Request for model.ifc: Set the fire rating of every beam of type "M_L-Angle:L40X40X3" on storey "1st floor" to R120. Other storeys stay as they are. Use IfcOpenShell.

First a look at what the model holds.

```python
import ifcopenshell
import ifcopenshell.util.element

model = ifcopenshell.open("model.ifc")
print(model.schema)
storey = next(s for s in model.by_type("IfcBuildingStorey") if s.Name == "1st floor")
beams = [e for e in ifcopenshell.util.element.get_decomposition(storey) if e.is_a("IfcBeam")]
seen = {}
for e in beams:
    element_type = ifcopenshell.util.element.get_type(e)
    key = (element_type.Name if element_type != e and element_type else None, ifcopenshell.util.element.get_pset(e, "Pset_BeamCommon", "FireRating"))
    seen[key] = seen.get(key, 0) + 1
for (name, value), count in sorted(seen.items(), key=str):
    print(count, "x", name, "|", value)
```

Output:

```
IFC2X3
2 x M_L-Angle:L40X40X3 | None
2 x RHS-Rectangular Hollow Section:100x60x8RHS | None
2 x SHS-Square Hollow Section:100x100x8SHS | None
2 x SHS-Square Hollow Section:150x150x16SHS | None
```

```python
import ifcopenshell
import ifcopenshell.api.pset
import ifcopenshell.util.element

model = ifcopenshell.open("model.ifc")

storey = next(s for s in model.by_type("IfcBuildingStorey") if s.Name == "1st floor")
beams = [e for e in ifcopenshell.util.element.get_decomposition(storey) if e.is_a("IfcBeam")]

count = 0
for e in beams:
    element_type = ifcopenshell.util.element.get_type(e)
    if element_type in (None, e) or element_type.Name != "M_L-Angle:L40X40X3":
        continue
    # add_pset returns the element's existing set when there is one.
    pset = ifcopenshell.api.pset.add_pset(model, product=e, name="Pset_BeamCommon")
    ifcopenshell.api.pset.edit_pset(model, pset=pset, properties={"FireRating": "R120"})
    count += 1

print(count, "beams updated")

model.write("model_updated.ifc")
```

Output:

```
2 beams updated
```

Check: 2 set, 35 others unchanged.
